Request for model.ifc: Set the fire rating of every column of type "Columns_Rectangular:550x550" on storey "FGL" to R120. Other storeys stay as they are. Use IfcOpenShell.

First a look at what the model holds.

```python
import ifcopenshell
import ifcopenshell.util.element

model = ifcopenshell.open("model.ifc")
print(model.schema)
storey = next(s for s in model.by_type("IfcBuildingStorey") if s.Name == "FGL")
columns = [e for e in ifcopenshell.util.element.get_decomposition(storey) if e.is_a("IfcColumn")]
seen = {}
for e in columns:
    element_type = ifcopenshell.util.element.get_type(e)
    key = (element_type.Name if element_type != e and element_type else None, ifcopenshell.util.element.get_pset(e, "Pset_ColumnCommon", "FireRating"))
    seen[key] = seen.get(key, 0) + 1
for (name, value), count in sorted(seen.items(), key=str):
    print(count, "x", name, "|", value)
```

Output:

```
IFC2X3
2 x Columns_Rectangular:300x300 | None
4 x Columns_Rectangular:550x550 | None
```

```python
import ifcopenshell
import ifcopenshell.api.pset
import ifcopenshell.util.element

model = ifcopenshell.open("model.ifc")

storey = next(s for s in model.by_type("IfcBuildingStorey") if s.Name == "FGL")
columns = [e for e in ifcopenshell.util.element.get_decomposition(storey) if e.is_a("IfcColumn")]

count = 0
for e in columns:
    element_type = ifcopenshell.util.element.get_type(e)
    if element_type in (None, e) or element_type.Name != "Columns_Rectangular:550x550":
        continue
    # add_pset returns the element's existing set when there is one.
    pset = ifcopenshell.api.pset.add_pset(model, product=e, name="Pset_ColumnCommon")
    ifcopenshell.api.pset.edit_pset(model, pset=pset, properties={"FireRating": "R120"})
    count += 1

print(count, "columns updated")

model.write("model_edited.ifc")
```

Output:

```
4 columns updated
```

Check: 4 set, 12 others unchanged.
